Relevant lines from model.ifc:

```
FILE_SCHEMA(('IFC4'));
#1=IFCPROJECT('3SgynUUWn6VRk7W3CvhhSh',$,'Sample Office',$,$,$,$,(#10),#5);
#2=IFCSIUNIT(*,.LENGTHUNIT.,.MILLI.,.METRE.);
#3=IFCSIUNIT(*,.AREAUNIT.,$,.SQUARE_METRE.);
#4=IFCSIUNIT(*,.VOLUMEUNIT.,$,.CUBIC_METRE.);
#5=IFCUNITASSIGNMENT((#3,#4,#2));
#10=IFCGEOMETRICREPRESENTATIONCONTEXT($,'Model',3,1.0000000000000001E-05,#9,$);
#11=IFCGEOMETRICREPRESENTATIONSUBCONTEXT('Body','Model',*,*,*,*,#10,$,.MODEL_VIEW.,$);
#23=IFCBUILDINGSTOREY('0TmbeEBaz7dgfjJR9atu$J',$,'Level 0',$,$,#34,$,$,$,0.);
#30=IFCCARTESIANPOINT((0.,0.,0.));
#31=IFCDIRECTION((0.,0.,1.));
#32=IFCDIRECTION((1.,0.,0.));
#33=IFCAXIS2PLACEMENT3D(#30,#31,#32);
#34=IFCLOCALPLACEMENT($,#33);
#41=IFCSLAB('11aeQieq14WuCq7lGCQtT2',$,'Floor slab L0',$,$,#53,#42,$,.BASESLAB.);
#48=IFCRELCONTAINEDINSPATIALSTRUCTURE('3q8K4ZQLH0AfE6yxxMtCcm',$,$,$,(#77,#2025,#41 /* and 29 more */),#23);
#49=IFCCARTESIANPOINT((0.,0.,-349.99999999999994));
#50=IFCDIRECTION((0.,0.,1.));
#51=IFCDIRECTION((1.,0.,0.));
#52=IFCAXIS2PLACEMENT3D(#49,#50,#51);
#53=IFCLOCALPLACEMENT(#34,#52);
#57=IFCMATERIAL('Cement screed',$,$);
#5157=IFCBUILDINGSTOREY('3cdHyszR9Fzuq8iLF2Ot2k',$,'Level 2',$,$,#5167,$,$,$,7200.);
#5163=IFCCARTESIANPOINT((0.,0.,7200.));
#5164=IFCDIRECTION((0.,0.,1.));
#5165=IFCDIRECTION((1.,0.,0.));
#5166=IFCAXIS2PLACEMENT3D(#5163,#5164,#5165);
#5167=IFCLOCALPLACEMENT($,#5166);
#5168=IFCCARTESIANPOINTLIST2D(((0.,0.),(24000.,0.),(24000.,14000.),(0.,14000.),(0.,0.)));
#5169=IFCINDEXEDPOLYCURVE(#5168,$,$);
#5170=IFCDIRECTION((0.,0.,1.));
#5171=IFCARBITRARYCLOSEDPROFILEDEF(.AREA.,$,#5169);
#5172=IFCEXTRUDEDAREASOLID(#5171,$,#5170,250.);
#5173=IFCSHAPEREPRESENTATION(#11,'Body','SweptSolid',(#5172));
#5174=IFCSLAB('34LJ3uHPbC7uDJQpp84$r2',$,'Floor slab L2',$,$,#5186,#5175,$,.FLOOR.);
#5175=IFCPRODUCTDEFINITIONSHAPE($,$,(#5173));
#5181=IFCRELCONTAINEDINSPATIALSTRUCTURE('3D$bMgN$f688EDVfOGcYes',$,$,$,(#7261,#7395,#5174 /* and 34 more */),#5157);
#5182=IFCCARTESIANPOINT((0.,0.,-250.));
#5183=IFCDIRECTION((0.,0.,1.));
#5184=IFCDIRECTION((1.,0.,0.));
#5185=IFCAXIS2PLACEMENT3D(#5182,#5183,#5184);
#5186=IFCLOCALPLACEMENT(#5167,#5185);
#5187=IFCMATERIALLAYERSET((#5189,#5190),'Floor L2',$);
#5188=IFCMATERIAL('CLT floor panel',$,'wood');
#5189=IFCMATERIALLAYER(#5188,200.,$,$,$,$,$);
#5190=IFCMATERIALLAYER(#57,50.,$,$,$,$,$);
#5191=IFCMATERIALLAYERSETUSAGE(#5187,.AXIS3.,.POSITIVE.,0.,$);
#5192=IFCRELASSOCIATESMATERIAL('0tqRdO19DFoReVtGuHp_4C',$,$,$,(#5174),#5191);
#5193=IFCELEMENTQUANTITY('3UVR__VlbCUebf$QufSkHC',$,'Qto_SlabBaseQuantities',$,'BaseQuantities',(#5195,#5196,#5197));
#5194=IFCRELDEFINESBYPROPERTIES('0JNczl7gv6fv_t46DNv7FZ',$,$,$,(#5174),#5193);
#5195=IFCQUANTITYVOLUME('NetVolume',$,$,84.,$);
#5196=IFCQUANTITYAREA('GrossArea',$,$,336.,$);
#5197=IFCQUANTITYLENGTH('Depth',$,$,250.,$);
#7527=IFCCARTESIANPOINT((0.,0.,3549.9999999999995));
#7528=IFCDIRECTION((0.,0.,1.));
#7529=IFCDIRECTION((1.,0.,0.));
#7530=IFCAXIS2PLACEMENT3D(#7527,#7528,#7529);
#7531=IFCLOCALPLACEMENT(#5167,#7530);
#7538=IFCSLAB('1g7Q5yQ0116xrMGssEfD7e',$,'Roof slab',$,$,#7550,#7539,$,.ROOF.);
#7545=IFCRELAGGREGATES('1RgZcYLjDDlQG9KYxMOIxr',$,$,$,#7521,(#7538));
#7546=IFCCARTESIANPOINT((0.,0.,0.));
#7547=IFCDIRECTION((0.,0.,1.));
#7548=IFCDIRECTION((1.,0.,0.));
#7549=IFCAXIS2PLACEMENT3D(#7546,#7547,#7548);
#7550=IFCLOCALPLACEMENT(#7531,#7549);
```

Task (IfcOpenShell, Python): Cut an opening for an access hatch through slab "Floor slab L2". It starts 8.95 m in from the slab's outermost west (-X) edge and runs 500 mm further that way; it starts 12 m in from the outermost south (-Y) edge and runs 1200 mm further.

```python
import numpy as np
import ifcopenshell
import ifcopenshell.api.feature
import ifcopenshell.api.geometry
import ifcopenshell.api.pset
import ifcopenshell.api.root
import ifcopenshell.geom
import ifcopenshell.util.element
import ifcopenshell.util.placement
import ifcopenshell.util.representation
import ifcopenshell.util.shape
import ifcopenshell.util.unit

model = ifcopenshell.open("model.ifc")
unit_scale = ifcopenshell.util.unit.calculate_unit_scale(model)
volume_scale = ifcopenshell.util.unit.calculate_unit_scale(model, "VOLUMEUNIT")
settings = ifcopenshell.geom.settings()


def volume(element):
    """Net volume in cubic metres, openings subtracted."""
    shape = ifcopenshell.geom.create_shape(settings, element)
    return ifcopenshell.util.shape.get_volume(shape.geometry)


slab = model.by_guid("34LJ3uHPbC7uDJQpp84$r2")
before = volume(slab)

# Extent in the slab's own axes, in metres. The edges named are its -X and -Y sides.
slab_shape = ifcopenshell.geom.create_shape(settings, slab)
vertices = ifcopenshell.util.shape.get_vertices(slab_shape.geometry)
x_min, y_min, bottom = vertices.min(axis=0)
top = vertices[:, 2].max()

opening = ifcopenshell.api.root.create_entity(model, ifc_class="IfcOpeningElement", name="Access hatch opening", predefined_type="OPENING")
context = ifcopenshell.util.representation.get_context(model, "Model", "Body", "MODEL_VIEW")
width, depth = 0.5, 1.2
outline = [(0.0, 0.0), (width, 0.0), (width, depth), (0.0, depth), (0.0, 0.0)]
# Overshoot both faces by 50 mm so the cut is clean.
shape = ifcopenshell.api.geometry.add_slab_representation(
    model, context=context, depth=top - bottom + 0.1, polyline=outline
)
ifcopenshell.api.geometry.assign_representation(model, product=opening, representation=shape)

matrix = ifcopenshell.util.placement.get_local_placement(slab.ObjectPlacement)
matrix[:, 3] = matrix @ np.append(np.array([x_min + 8.95, y_min + 12, bottom - 0.05]) / unit_scale, 1.0)
ifcopenshell.api.geometry.edit_object_placement(model, product=opening, matrix=matrix, is_si=False)
ifcopenshell.api.feature.add_feature(model, feature=opening, element=slab)

after = volume(slab)

# Update the slab's stored quantities.
qto = model.by_id(ifcopenshell.util.element.get_pset(slab, "Qto_SlabBaseQuantities", should_inherit=False)["id"])
ifcopenshell.api.pset.edit_qto(model, qto=qto, properties={"NetVolume": after / volume_scale})

print(f"slab volume {before:.3f} -> {after:.3f} m3")

model.write("model_rev.ifc")
```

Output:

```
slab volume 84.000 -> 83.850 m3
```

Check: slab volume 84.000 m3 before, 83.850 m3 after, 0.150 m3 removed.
